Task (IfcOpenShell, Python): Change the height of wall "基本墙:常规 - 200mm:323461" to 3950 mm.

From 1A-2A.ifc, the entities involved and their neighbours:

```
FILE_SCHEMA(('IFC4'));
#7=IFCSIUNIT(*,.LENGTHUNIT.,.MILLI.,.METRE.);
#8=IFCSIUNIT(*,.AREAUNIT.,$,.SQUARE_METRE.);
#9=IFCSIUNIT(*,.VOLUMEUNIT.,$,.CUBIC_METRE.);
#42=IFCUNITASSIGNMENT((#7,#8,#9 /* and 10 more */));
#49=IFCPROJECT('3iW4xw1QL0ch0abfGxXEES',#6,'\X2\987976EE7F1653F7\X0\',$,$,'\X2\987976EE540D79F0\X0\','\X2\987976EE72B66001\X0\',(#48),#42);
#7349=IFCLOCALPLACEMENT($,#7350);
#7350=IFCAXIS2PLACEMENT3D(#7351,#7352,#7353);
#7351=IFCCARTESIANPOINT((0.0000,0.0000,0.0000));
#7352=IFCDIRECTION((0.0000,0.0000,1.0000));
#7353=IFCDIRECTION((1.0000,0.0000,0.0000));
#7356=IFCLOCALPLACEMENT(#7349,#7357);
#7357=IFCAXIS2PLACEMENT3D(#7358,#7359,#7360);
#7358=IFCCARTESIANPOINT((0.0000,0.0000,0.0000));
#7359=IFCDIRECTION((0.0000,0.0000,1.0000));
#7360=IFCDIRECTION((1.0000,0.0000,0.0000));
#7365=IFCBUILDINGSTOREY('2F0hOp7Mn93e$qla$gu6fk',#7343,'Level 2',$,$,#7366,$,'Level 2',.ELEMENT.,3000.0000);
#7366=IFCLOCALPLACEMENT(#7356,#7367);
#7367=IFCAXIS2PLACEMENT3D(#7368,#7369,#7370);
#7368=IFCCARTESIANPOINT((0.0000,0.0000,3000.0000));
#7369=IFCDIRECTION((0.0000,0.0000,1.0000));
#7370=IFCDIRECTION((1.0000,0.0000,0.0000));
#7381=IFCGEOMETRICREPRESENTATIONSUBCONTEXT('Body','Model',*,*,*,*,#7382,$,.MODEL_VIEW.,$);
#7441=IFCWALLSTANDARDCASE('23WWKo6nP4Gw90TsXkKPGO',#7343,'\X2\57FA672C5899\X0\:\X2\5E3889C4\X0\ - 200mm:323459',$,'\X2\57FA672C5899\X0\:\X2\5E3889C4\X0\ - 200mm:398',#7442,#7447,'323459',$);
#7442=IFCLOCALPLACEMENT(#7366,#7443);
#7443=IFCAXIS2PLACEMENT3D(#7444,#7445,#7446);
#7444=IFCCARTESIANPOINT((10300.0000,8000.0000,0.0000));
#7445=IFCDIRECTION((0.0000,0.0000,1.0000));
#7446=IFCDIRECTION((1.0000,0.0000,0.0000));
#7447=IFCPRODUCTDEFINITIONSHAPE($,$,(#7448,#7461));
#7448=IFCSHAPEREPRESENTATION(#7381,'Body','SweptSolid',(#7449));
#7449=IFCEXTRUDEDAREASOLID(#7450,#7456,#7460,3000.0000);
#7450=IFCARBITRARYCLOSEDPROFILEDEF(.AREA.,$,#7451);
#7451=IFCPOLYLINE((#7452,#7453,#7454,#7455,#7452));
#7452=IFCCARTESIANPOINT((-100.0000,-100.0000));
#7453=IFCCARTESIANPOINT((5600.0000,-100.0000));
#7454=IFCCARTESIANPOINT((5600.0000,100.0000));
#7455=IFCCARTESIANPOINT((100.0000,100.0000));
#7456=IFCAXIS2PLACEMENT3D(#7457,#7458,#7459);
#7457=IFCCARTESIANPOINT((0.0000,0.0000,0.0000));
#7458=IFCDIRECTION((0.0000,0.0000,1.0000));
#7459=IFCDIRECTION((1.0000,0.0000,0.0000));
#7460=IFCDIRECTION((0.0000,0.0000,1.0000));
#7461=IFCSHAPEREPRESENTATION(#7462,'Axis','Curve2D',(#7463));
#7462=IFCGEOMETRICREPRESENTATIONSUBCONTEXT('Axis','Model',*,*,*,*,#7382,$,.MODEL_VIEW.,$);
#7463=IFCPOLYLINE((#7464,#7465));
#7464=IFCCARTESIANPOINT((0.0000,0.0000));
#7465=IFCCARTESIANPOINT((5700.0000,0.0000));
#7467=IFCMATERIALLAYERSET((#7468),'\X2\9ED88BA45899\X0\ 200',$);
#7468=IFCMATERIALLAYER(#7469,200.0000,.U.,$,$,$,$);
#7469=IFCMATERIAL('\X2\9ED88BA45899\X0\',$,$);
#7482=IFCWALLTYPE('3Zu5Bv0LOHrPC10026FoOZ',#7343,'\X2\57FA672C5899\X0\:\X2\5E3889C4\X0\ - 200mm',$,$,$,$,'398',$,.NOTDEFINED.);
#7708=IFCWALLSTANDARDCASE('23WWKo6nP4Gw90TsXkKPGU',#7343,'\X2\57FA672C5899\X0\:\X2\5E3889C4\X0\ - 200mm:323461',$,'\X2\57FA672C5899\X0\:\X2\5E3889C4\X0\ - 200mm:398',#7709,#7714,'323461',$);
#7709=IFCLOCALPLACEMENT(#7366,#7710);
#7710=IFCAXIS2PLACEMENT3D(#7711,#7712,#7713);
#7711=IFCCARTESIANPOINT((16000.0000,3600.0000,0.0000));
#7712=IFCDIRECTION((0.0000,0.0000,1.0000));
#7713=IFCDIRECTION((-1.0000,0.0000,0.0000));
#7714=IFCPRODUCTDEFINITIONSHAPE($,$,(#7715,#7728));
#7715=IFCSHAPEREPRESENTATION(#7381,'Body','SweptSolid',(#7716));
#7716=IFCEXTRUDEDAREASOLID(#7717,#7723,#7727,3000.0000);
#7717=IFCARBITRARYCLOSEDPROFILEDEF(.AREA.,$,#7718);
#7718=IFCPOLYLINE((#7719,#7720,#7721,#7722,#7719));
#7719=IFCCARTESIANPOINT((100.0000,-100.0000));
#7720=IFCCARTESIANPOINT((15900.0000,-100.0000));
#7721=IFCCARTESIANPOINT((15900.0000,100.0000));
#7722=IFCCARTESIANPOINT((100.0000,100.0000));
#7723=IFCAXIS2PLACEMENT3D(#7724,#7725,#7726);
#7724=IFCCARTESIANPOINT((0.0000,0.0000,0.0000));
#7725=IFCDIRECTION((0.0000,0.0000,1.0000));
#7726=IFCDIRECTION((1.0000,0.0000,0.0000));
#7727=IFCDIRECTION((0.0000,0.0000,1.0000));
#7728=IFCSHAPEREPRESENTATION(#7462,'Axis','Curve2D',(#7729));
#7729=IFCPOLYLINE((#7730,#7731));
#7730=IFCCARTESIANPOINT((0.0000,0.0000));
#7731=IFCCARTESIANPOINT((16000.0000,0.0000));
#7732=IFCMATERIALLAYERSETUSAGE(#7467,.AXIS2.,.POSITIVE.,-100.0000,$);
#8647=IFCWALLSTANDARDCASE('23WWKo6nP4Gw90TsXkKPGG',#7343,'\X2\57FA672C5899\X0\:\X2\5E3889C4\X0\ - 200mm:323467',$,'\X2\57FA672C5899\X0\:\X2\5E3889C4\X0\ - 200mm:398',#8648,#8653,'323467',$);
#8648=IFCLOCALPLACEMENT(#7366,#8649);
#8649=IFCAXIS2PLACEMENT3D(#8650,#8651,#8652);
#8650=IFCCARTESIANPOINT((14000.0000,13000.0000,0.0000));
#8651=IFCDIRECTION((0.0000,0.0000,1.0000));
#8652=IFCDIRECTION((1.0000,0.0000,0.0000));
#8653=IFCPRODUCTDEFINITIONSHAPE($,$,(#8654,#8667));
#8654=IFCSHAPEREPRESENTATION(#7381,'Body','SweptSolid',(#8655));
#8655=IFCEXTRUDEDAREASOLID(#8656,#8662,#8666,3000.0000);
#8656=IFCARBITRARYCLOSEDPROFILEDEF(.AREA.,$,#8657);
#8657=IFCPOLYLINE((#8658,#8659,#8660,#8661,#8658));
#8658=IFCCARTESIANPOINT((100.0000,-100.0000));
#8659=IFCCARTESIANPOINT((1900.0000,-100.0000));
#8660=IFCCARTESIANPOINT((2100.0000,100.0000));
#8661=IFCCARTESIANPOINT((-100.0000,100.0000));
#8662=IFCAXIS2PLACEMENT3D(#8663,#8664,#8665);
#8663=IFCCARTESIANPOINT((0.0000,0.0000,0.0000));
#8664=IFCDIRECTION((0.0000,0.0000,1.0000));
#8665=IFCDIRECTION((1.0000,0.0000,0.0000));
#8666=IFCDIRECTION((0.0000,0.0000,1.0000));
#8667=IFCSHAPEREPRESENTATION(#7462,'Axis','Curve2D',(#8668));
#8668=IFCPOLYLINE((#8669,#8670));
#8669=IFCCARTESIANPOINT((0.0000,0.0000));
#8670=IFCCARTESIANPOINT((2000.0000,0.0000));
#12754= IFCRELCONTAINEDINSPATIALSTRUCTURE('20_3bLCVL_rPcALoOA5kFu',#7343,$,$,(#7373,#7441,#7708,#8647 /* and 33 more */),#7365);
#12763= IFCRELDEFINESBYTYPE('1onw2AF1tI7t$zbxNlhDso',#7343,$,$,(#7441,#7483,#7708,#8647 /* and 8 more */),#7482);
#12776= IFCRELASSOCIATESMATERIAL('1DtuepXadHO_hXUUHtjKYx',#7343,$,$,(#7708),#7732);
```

```python
import ifcopenshell
import ifcopenshell.geom
import ifcopenshell.util.representation
import ifcopenshell.util.shape
import ifcopenshell.util.unit

model = ifcopenshell.open("1A-2A.ifc")
unit_scale = ifcopenshell.util.unit.calculate_unit_scale(model)
settings = ifcopenshell.geom.settings()


def volume(element):
    """Net volume in cubic metres, openings subtracted."""
    shape = ifcopenshell.geom.create_shape(settings, element)
    return ifcopenshell.util.shape.get_volume(shape.geometry)


wall = model.by_guid("23WWKo6nP4Gw90TsXkKPGU")
before = volume(wall)

body = ifcopenshell.util.representation.get_representation(wall, "Model", "Body")
solid = body.Items[0]
old_height = solid.Depth
solid.Depth = 3.95 / unit_scale
after = volume(wall)

print(f"height {old_height:g} -> {solid.Depth:g}, volume {before:.3f} -> {after:.3f} m3")

model.write("1A-2A_v2.ifc")
```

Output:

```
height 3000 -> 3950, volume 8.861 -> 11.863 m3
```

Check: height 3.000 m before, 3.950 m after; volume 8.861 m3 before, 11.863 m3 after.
